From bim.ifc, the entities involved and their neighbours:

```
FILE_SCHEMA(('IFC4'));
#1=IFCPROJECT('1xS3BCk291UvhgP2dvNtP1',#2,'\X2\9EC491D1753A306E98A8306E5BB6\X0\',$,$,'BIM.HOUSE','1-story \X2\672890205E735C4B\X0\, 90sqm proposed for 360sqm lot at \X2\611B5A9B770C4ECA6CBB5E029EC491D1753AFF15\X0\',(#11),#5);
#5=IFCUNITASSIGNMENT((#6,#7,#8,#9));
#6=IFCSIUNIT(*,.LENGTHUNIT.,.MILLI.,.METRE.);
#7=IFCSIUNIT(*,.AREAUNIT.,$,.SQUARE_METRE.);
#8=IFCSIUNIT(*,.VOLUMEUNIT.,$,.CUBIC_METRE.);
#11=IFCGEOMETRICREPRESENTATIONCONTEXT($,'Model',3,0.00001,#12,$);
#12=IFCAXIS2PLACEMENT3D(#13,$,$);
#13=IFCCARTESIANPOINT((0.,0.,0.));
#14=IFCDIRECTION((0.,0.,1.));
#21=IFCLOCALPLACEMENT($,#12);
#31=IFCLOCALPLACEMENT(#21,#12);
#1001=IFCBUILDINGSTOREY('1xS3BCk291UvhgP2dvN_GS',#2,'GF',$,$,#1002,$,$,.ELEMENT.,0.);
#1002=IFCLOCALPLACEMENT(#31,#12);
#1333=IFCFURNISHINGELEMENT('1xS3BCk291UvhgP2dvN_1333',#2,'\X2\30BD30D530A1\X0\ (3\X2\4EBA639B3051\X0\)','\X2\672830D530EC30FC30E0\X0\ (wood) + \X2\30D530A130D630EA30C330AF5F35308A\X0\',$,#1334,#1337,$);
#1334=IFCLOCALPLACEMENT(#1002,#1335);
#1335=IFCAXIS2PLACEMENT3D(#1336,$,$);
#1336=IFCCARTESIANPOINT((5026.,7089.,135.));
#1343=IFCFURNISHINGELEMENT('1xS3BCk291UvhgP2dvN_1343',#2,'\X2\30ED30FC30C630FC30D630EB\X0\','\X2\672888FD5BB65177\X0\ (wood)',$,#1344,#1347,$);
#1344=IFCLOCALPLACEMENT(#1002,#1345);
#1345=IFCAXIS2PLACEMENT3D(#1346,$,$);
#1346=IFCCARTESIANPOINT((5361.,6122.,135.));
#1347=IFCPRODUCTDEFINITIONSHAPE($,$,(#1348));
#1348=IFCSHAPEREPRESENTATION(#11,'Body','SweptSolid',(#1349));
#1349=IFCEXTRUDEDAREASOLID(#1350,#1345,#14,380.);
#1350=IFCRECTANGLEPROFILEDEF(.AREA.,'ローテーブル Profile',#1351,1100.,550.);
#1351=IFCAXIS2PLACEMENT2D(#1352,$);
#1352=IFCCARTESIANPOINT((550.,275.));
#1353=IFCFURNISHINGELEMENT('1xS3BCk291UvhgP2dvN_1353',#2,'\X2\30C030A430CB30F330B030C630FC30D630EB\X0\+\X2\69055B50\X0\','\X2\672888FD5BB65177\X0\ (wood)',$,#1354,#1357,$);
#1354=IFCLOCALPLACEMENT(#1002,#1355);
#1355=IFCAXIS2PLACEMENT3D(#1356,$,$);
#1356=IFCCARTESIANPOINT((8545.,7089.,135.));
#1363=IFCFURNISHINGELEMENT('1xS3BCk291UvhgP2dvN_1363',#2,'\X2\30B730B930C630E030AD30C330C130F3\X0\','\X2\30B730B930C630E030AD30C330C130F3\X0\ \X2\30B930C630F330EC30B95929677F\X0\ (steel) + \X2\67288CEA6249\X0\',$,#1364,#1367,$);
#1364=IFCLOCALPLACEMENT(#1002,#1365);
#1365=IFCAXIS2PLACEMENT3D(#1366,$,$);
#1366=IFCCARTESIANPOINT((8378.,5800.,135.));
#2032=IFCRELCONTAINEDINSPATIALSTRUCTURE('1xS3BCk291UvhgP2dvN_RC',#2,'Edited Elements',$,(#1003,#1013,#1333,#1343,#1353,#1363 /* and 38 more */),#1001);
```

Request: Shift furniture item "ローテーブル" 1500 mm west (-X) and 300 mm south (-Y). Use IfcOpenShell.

```python
import ifcopenshell
import ifcopenshell.api.geometry
import ifcopenshell.util.placement
import ifcopenshell.util.unit

model = ifcopenshell.open("bim.ifc")
unit_scale = ifcopenshell.util.unit.calculate_unit_scale(model)

item = model.by_id(1343)
matrix = ifcopenshell.util.placement.get_local_placement(item.ObjectPlacement)
matrix[0, 3] -= 1.5 / unit_scale
matrix[1, 3] -= 0.3 / unit_scale
ifcopenshell.api.geometry.edit_object_placement(model, product=item, matrix=matrix, is_si=False)

print(ifcopenshell.util.placement.get_local_placement(item.ObjectPlacement).round(3) + 0.0)

model.write("bim_updated.ifc")
```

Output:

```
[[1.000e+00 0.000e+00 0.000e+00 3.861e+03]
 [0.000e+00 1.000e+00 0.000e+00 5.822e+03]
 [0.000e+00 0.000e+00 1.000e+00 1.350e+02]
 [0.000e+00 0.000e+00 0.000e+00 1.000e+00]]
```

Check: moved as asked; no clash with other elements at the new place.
